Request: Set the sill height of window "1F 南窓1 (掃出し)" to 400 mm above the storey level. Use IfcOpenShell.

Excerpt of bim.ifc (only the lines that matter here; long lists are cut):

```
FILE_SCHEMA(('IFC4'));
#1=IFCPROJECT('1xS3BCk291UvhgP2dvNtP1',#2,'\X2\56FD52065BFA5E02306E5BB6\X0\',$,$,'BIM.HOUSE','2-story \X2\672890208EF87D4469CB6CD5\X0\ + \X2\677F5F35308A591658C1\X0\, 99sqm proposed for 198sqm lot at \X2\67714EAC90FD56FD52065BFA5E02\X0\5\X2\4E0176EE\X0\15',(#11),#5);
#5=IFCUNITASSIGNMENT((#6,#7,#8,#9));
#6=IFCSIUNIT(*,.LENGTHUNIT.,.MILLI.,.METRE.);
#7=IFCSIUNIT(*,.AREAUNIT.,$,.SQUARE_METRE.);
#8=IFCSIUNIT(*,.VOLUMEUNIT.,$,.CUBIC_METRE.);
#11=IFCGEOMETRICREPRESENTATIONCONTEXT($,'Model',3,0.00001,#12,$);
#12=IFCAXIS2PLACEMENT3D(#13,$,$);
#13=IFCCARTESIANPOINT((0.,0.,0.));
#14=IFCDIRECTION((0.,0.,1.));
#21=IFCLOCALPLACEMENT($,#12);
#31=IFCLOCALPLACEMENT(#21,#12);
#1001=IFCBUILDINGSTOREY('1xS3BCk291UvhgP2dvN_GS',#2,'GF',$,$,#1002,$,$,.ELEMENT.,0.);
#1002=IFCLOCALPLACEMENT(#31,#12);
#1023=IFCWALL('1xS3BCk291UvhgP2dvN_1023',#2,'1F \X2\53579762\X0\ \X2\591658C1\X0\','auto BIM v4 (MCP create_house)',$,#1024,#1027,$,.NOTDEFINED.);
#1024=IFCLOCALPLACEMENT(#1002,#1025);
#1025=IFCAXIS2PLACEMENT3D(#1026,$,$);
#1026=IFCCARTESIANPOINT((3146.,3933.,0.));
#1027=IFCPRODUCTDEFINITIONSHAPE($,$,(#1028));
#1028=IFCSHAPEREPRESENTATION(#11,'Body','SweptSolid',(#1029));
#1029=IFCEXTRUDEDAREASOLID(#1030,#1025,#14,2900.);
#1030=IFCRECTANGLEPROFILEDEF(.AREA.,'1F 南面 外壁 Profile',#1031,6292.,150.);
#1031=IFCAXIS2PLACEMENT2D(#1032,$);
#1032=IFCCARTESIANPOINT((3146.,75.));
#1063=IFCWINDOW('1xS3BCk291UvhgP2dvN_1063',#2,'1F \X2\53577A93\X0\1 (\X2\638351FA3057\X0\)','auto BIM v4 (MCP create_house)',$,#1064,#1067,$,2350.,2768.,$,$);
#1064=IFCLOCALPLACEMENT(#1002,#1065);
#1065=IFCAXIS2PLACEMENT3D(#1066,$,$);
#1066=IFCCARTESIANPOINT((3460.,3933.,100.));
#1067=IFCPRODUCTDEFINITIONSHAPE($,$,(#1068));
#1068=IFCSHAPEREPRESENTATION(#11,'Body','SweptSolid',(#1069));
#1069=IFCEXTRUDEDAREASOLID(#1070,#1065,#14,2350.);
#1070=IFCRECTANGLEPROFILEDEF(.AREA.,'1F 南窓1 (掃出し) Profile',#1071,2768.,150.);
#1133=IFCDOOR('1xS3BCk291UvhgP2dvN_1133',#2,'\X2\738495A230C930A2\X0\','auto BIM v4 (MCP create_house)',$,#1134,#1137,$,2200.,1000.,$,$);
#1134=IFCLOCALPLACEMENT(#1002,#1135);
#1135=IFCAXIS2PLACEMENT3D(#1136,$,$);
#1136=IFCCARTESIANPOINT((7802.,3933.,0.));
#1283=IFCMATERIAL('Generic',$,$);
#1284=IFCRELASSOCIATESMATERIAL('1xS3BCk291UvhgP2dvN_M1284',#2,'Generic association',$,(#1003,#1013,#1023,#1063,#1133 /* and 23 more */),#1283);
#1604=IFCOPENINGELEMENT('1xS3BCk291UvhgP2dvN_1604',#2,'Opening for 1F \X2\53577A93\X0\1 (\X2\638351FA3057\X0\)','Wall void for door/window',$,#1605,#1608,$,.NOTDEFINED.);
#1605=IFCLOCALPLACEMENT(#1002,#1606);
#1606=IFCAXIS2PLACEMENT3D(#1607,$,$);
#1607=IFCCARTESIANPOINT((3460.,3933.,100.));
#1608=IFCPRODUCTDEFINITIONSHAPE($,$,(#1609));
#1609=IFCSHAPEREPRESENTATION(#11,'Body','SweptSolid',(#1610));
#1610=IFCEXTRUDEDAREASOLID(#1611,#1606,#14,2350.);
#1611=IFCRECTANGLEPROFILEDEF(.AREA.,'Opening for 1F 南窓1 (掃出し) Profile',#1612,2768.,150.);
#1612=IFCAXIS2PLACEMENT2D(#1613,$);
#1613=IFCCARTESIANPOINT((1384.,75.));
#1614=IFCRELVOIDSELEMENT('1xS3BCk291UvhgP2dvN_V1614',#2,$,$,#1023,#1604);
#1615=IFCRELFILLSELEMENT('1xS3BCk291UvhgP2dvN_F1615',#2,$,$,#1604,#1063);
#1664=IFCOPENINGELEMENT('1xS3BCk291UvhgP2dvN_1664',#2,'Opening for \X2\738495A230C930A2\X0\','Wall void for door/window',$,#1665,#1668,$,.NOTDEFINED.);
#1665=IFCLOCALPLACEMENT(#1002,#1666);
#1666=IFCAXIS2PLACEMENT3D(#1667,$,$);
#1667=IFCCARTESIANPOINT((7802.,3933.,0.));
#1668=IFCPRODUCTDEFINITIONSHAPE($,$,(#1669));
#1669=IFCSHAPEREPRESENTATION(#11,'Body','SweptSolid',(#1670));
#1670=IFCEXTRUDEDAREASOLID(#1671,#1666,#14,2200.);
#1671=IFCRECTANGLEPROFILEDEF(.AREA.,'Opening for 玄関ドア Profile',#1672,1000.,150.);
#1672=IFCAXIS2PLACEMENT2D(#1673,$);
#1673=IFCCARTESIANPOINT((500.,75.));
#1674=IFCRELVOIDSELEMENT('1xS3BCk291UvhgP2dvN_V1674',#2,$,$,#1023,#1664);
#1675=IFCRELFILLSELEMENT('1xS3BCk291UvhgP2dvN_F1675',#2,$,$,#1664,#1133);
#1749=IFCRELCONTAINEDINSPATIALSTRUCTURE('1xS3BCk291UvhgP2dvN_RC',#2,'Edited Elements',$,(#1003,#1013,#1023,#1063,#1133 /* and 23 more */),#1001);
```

```python
import numpy as np
import ifcopenshell
import ifcopenshell.api.geometry
import ifcopenshell.geom
import ifcopenshell.util.element
import ifcopenshell.util.placement
import ifcopenshell.util.shape
import ifcopenshell.util.unit

model = ifcopenshell.open("bim.ifc")
unit_scale = ifcopenshell.util.unit.calculate_unit_scale(model)

window = model.by_guid("1xS3BCk291UvhgP2dvN_1063")
opening = window.FillsVoids[0].RelatingOpeningElement
storey = ifcopenshell.util.element.get_container(window, ifc_class="IfcBuildingStorey")
level = ifcopenshell.util.placement.get_local_placement(storey.ObjectPlacement)[2, 3]

# The opening's origin need not be at the sill, so measure its lowest point.
shape = ifcopenshell.geom.create_shape(ifcopenshell.geom.settings(), opening)
bottom = ifcopenshell.util.shape.get_shape_bottom_elevation(shape, shape.geometry) / unit_scale
dz = level + 400.0 - bottom

shift = np.array([0.0, 0.0, dz])
# The window is not placed relative to its opening, so move both.
for product in (opening, window):
    matrix = ifcopenshell.util.placement.get_local_placement(product.ObjectPlacement)
    matrix[:3, 3] += shift
    ifcopenshell.api.geometry.edit_object_placement(model, product=product, matrix=matrix, is_si=False)

print(f"moved by {dz * unit_scale:+.3f} m")

model.write("bim_rev.ifc")
```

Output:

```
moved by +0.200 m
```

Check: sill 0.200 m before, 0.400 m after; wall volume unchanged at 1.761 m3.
